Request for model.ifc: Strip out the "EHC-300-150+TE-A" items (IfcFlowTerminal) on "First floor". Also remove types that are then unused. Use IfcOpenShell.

First a look at what the model holds.

```python
import ifcopenshell
import ifcopenshell.util.element

model = ifcopenshell.open("model.ifc")
print(model.schema)
storey = next(s for s in model.by_type("IfcBuildingStorey") if s.Name == "First floor")
terminals = [e for e in ifcopenshell.util.element.get_decomposition(storey) if e.is_a("IfcFlowTerminal")]
seen = {}
for e in terminals:
    element_type = ifcopenshell.util.element.get_type(e)
    name = element_type.Name if element_type not in (None, e) else None
    seen[name] = seen.get(name, 0) + 1
for name, count in sorted(seen.items(), key=str):
    print(count, "x", name)
```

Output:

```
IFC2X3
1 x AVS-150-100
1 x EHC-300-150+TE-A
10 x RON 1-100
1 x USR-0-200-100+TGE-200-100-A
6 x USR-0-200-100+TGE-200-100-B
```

```python
import ifcopenshell
import ifcopenshell.api.root
import ifcopenshell.util.element

model = ifcopenshell.open("model.ifc")

storey = next(s for s in model.by_type("IfcBuildingStorey") if s.Name == "First floor")
terminals = [e for e in ifcopenshell.util.element.get_decomposition(storey) if e.is_a("IfcFlowTerminal")]
targets = [e for e in terminals if (t := ifcopenshell.util.element.get_type(e)) not in (None, e) and t.Name == "EHC-300-150+TE-A"]
types = {ifcopenshell.util.element.get_type(e) for e in targets} - {None, *targets}

for e in targets:
    ifcopenshell.api.root.remove_product(model, product=e)
print(len(targets), "removed")

unused = [t for t in types if not ifcopenshell.util.element.get_types(t)]
for t in unused:
    ifcopenshell.api.root.remove_product(model, product=t)
print(len(unused), "unused types removed")

model.write("model_v2.ifc")
```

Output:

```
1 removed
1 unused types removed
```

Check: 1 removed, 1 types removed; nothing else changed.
